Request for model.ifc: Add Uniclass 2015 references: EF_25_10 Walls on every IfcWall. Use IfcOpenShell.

First a look at what the model holds.

```python
import ifcopenshell

model = ifcopenshell.open("model.ifc")
print(model.schema)
print("classifications:", [c.Name for c in model.by_type("IfcClassification")])
for ifc_class in ("IfcDoor", "IfcRoof", "IfcStair", "IfcWall", "IfcWindow"):
    print(ifc_class, len(model.by_type(ifc_class)))
```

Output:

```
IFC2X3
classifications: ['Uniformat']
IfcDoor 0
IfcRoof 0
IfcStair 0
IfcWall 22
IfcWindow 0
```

```python
import ifcopenshell
import ifcopenshell.api.classification

model = ifcopenshell.open("model.ifc")

# IFC2X3 requires Source and Edition and has no link from the project to the system.
system = model.create_entity("IfcClassification", Source="NBS", Edition="2015", Name="Uniclass 2015")

codes = {
    "IfcWall": ("EF_25_10", "Walls"),
}
for ifc_class, (code, name) in codes.items():
    products = model.by_type(ifc_class)
    ifcopenshell.api.classification.add_reference(
        model, products=products, classification=system, identification=code, name=name
    )
    print(code, len(products))

model.write("model-out.ifc")
```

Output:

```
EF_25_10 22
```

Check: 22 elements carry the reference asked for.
